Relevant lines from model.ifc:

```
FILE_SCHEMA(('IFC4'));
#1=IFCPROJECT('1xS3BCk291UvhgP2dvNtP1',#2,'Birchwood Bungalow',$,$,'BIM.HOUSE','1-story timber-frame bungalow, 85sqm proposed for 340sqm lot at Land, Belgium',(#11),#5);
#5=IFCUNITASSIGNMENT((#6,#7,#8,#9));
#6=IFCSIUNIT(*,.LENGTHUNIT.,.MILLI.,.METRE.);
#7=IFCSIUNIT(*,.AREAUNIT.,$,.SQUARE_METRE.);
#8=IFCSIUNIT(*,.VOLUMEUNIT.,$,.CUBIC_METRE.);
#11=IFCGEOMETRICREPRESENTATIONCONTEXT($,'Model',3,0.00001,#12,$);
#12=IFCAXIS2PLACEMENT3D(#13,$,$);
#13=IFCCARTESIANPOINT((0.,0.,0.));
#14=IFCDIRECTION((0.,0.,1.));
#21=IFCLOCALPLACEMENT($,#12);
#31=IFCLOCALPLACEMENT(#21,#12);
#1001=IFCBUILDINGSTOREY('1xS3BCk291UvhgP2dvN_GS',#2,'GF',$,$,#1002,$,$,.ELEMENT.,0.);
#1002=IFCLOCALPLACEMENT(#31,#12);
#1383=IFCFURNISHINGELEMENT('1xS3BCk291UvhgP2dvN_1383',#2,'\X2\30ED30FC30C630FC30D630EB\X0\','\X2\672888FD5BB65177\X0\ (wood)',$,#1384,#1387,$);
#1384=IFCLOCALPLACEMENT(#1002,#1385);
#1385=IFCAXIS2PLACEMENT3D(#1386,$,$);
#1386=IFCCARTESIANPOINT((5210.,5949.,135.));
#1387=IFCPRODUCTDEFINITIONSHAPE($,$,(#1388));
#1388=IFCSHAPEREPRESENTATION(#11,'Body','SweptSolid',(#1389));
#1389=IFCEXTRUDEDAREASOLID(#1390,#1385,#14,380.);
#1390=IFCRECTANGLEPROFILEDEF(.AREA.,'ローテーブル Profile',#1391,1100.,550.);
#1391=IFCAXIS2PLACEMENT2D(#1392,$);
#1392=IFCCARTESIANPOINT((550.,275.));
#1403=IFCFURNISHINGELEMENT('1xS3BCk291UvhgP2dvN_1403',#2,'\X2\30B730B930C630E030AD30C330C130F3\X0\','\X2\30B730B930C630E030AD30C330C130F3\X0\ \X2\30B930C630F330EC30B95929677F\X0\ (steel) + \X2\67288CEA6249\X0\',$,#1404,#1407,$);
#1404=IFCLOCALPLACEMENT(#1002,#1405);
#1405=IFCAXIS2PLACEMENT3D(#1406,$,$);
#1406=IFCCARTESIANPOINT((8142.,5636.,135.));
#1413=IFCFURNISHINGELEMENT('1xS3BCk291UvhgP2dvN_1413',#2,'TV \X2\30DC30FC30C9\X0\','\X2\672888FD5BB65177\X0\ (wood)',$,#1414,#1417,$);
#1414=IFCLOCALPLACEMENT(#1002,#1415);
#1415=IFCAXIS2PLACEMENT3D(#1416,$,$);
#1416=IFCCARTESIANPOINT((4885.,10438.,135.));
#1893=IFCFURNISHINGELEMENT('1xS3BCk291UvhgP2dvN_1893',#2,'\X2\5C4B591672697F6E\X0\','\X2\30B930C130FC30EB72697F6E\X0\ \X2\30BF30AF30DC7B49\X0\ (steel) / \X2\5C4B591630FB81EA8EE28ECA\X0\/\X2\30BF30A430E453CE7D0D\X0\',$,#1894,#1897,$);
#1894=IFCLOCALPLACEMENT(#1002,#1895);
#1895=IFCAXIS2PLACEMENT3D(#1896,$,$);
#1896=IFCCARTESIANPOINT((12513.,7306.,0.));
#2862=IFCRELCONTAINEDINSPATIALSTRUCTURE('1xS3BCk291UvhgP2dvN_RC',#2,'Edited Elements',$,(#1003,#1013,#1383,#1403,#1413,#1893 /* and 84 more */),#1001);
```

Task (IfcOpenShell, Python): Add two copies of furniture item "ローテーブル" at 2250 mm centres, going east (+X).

```python
import numpy as np
import ifcopenshell
import ifcopenshell.api.geometry
import ifcopenshell.api.root
import ifcopenshell.util.element
import ifcopenshell.util.placement
import ifcopenshell.util.unit

model = ifcopenshell.open("model.ifc")
unit_scale = ifcopenshell.util.unit.calculate_unit_scale(model)


def reuse_history(source, copy):
    """copy_class also copies each property set's owner history, people and application; keep the originals."""
    for rel in copy.IsDefinedBy:
        if rel.is_a("IfcRelDefinesByProperties") and (history := rel.RelatingPropertyDefinition.OwnerHistory):
            rel.RelatingPropertyDefinition.OwnerHistory = source.OwnerHistory
            ifcopenshell.util.element.remove_deep2(model, history)


source = model.by_id(1383)
base = ifcopenshell.util.placement.get_local_placement(source.ObjectPlacement)
step = np.array([1.0, 0.0, 0.0]) * 2.25 / unit_scale

for i in range(1, 3):
    copy = ifcopenshell.api.root.copy_class(model, product=source)
    copy.Representation = ifcopenshell.util.element.copy_deep(
        model, source.Representation, exclude=["IfcGeometricRepresentationContext", "IfcRepresentationMap"]
    )
    reuse_history(source, copy)
    matrix = base.copy()
    matrix[:3, 3] += i * step
    print("added at", matrix[:3, 3].round(3) + 0.0)
    ifcopenshell.api.geometry.edit_object_placement(model, product=copy, matrix=matrix, is_si=False)

model.write("model_v2.ifc")
```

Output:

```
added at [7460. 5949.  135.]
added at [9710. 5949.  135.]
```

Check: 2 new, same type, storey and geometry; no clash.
